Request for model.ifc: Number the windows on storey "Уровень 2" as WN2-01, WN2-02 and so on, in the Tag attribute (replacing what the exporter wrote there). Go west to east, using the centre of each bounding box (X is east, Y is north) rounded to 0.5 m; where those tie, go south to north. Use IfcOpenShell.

First a look at what the model holds.

```python
import ifcopenshell
import ifcopenshell.util.element
import ifcopenshell.util.placement

model = ifcopenshell.open("model.ifc")
print(model.schema)
storey = next(s for s in model.by_type("IfcBuildingStorey") if s.Name == "Уровень 2")
windows = [e for e in ifcopenshell.util.element.get_decomposition(storey) if e.is_a("IfcWindow")]
for e in sorted(windows, key=lambda e: e.id()):
    origin = ifcopenshell.util.placement.get_local_placement(e.ObjectPlacement)[:3, 3]
    print(e.id(), e.Tag, e.Name, origin.round(2) + 0.0, sep=" | ")
```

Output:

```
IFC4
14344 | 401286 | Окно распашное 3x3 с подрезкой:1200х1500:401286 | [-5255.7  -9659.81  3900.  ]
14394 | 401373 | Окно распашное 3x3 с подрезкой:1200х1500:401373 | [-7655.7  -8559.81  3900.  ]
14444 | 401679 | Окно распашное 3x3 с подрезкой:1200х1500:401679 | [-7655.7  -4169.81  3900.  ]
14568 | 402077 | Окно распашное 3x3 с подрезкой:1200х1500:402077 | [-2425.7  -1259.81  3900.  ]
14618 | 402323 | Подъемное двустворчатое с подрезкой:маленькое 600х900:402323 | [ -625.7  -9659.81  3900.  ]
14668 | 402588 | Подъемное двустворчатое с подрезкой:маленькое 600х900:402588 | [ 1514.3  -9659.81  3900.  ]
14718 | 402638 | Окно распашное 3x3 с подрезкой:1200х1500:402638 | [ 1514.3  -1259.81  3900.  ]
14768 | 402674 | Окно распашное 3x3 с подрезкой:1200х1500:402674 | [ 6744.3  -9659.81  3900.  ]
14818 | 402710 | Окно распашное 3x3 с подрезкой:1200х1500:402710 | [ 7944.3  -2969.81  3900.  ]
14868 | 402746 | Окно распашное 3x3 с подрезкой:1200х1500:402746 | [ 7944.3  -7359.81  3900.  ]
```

```python
import ifcopenshell
import ifcopenshell.geom
import ifcopenshell.util.element
import ifcopenshell.util.shape

model = ifcopenshell.open("model.ifc")
settings = ifcopenshell.geom.settings()
settings.set("use-world-coords", True)


def centre(element):
    shape = ifcopenshell.geom.create_shape(settings, element)
    return ifcopenshell.util.shape.get_bbox_centroid(shape.geometry)


storey = next(s for s in model.by_type("IfcBuildingStorey") if s.Name == "Уровень 2")
windows = [e for e in ifcopenshell.util.element.get_decomposition(storey) if e.is_a("IfcWindow")]

# Insertion points can sit at a corner or the storey origin, so sort by the geometry (in metres).
centres = {e: centre(e) for e in windows}
windows.sort(key=lambda e: (round(centres[e][0] / 0.5), centres[e][1]))

for i, e in enumerate(windows, start=1):
    number = f"WN2-{i:02d}"
    e.Tag = number
    print(e.id(), number)

model.write("model_v2.ifc")
```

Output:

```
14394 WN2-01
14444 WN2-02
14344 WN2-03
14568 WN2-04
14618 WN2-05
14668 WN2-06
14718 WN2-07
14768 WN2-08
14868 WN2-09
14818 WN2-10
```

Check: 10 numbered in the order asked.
